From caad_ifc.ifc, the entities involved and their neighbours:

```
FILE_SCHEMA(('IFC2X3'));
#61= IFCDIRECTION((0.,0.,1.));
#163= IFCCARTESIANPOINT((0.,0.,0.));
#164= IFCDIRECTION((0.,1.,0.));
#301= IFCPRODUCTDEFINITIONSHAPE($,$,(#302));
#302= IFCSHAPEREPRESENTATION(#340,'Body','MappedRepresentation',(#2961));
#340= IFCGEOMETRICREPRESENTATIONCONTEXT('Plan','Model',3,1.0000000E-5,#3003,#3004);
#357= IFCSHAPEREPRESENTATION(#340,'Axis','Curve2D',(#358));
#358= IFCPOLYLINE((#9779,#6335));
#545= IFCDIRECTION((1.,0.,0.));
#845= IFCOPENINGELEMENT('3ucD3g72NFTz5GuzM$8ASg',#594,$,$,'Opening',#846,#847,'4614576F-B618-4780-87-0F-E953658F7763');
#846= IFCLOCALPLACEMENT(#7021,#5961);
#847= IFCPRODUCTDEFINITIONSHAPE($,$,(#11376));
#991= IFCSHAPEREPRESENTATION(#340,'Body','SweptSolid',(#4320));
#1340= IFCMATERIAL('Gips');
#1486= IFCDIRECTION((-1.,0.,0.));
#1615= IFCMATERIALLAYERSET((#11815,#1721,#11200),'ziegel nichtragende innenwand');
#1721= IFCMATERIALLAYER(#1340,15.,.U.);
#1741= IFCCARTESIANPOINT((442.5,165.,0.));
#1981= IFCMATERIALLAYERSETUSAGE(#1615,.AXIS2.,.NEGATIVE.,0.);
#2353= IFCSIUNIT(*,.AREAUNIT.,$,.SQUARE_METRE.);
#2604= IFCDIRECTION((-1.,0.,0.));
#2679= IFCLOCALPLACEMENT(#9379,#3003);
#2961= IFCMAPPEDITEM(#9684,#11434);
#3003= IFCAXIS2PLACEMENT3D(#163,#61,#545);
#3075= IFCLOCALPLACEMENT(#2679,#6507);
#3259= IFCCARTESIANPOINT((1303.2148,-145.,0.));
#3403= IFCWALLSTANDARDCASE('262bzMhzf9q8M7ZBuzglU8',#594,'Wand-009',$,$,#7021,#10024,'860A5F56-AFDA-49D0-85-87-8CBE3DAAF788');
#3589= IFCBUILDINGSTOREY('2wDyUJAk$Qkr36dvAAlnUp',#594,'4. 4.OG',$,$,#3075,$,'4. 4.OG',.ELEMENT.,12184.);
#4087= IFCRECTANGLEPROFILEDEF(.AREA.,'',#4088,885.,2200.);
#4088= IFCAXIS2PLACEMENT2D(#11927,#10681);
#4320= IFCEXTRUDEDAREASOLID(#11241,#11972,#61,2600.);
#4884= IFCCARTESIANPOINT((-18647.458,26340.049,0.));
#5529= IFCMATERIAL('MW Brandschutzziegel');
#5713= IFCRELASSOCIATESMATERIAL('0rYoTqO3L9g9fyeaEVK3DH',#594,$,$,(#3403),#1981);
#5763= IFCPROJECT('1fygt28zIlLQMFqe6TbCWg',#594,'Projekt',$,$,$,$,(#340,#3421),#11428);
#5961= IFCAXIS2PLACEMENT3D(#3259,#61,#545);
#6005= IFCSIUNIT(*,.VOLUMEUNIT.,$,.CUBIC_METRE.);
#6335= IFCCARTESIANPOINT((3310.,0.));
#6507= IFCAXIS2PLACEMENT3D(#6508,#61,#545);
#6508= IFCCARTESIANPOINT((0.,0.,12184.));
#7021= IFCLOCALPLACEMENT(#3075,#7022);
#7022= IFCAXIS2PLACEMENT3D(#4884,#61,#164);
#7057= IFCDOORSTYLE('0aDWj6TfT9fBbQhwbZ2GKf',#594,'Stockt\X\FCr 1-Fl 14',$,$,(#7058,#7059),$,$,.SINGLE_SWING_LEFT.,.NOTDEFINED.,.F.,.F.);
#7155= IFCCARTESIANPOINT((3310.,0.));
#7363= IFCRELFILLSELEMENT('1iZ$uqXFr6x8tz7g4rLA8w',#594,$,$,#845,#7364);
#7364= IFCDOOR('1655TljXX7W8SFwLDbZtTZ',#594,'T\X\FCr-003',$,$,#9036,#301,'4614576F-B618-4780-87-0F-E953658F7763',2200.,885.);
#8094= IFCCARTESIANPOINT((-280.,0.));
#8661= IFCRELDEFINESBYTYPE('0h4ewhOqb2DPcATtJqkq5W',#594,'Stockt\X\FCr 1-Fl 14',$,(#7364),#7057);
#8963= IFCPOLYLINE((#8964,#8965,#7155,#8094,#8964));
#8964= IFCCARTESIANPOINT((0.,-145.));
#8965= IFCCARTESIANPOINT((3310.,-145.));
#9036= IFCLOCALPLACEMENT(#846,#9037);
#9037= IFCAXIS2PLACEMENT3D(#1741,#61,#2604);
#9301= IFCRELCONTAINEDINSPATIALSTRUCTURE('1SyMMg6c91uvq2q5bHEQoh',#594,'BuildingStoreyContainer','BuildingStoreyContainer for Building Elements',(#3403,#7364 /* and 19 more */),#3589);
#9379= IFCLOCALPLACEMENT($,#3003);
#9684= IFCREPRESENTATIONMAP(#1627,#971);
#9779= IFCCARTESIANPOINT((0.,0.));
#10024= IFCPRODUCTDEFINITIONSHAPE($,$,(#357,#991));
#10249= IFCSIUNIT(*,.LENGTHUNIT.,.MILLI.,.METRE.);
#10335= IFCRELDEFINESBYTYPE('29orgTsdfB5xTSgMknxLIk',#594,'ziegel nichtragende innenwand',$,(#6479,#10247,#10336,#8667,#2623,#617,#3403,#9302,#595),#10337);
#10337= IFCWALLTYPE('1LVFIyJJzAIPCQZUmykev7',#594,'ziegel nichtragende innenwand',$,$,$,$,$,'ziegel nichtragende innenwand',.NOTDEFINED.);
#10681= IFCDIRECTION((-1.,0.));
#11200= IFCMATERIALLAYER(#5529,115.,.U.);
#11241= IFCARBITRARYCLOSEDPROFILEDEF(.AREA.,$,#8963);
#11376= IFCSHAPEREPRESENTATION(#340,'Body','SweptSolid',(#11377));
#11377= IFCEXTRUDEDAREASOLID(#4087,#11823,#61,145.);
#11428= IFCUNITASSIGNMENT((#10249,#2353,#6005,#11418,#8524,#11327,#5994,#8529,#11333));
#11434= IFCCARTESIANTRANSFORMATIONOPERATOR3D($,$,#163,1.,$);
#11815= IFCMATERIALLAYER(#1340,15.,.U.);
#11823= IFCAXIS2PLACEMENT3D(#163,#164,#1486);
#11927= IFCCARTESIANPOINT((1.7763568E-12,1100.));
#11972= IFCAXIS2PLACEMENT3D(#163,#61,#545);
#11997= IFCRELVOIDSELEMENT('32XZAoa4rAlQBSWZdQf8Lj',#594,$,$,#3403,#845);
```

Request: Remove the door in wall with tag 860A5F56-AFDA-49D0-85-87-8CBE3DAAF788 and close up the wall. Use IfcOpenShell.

```python
import ifcopenshell
import ifcopenshell.api.feature
import ifcopenshell.api.root
import ifcopenshell.geom
import ifcopenshell.util.shape

model = ifcopenshell.open("caad_ifc.ifc")
settings = ifcopenshell.geom.settings()


def volume(element):
    """Net volume in cubic metres, openings subtracted."""
    shape = ifcopenshell.geom.create_shape(settings, element)
    return ifcopenshell.util.shape.get_volume(shape.geometry)


door = model.by_guid("1655TljXX7W8SFwLDbZtTZ")
opening = door.FillsVoids[0].RelatingOpeningElement
wall = opening.VoidsElements[0].RelatingBuildingElement
before = volume(wall)

ifcopenshell.api.root.remove_product(model, product=door)
ifcopenshell.api.feature.remove_feature(model, feature=opening)

after = volume(wall)

print(f"wall volume {before:.3f} -> {after:.3f} m3")

model.write("caad_ifc_edited.ifc")
```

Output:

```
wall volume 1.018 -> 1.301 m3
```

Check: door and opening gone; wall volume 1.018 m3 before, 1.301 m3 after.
